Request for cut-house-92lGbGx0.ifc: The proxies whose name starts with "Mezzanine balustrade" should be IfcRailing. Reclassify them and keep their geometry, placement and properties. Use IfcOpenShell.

First a look at what the model holds.

```python
import re

import ifcopenshell

model = ifcopenshell.open("cut-house-92lGbGx0.ifc")
print(model.schema)
seen = {}
for e in model.by_type("IfcBuildingElementProxy"):
    name = re.sub(r":\d+(:\d+)?$", "", e.Name or "")  # drop the element id that some exporters append
    seen[name] = seen.get(name, 0) + 1
for name, count in sorted(seen.items()):
    print(count, "x", name)
```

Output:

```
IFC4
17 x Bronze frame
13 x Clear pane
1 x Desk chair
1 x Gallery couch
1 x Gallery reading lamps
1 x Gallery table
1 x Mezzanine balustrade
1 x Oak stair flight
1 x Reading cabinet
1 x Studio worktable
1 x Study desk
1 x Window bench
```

```python
import ifcopenshell
import ifcopenshell.api.root

model = ifcopenshell.open("cut-house-92lGbGx0.ifc")

proxies = [e.id() for e in model.by_type("IfcBuildingElementProxy") if (e.Name or "").startswith("Mezzanine balustrade")]
for step_id in proxies:
    proxy = model.by_id(step_id)
    ifcopenshell.api.root.reassign_class(model, product=proxy, ifc_class="IfcRailing")

print(sum(model.by_id(i).is_a("IfcRailing") for i in proxies), "reclassified")

model.write("cut-house-92lGbGx0_rev.ifc")
```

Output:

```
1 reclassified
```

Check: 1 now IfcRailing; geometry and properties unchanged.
